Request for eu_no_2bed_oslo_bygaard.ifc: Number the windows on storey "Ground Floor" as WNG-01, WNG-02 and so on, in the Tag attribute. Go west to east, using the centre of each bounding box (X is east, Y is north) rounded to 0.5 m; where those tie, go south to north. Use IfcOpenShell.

First a look at what the model holds.

```python
import ifcopenshell
import ifcopenshell.util.element
import ifcopenshell.util.placement

model = ifcopenshell.open("eu_no_2bed_oslo_bygaard.ifc")
print(model.schema)
storey = next(s for s in model.by_type("IfcBuildingStorey") if s.Name == "Ground Floor")
windows = [e for e in ifcopenshell.util.element.get_decomposition(storey) if e.is_a("IfcWindow")]
for e in sorted(windows, key=lambda e: e.id()):
    origin = ifcopenshell.util.placement.get_local_placement(e.ObjectPlacement)[:3, 3]
    print(e.id(), e.Tag, e.Name, origin.round(2) + 0.0, sep=" | ")
```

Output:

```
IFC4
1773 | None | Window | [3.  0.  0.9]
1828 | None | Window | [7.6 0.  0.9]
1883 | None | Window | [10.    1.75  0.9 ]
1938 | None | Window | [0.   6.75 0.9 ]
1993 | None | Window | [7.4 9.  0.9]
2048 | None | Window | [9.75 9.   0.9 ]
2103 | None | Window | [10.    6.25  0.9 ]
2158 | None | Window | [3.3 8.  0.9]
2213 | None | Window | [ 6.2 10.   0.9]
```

```python
import ifcopenshell
import ifcopenshell.geom
import ifcopenshell.util.element
import ifcopenshell.util.shape

model = ifcopenshell.open("eu_no_2bed_oslo_bygaard.ifc")
settings = ifcopenshell.geom.settings()
settings.set("use-world-coords", True)


def centre(element):
    shape = ifcopenshell.geom.create_shape(settings, element)
    return ifcopenshell.util.shape.get_bbox_centroid(shape.geometry)


storey = next(s for s in model.by_type("IfcBuildingStorey") if s.Name == "Ground Floor")
windows = [e for e in ifcopenshell.util.element.get_decomposition(storey) if e.is_a("IfcWindow")]

# Insertion points can sit at a corner or the storey origin, so sort by the geometry (in metres).
centres = {e: centre(e) for e in windows}
windows.sort(key=lambda e: (round(centres[e][0] / 0.5), centres[e][1]))

for i, e in enumerate(windows, start=1):
    number = f"WNG-{i:02d}"
    e.Tag = number
    print(e.id(), number)

model.write("eu_no_2bed_oslo_bygaard_edited.ifc")
```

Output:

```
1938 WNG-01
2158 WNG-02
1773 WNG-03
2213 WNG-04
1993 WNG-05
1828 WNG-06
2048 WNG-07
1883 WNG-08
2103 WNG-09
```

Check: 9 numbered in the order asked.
